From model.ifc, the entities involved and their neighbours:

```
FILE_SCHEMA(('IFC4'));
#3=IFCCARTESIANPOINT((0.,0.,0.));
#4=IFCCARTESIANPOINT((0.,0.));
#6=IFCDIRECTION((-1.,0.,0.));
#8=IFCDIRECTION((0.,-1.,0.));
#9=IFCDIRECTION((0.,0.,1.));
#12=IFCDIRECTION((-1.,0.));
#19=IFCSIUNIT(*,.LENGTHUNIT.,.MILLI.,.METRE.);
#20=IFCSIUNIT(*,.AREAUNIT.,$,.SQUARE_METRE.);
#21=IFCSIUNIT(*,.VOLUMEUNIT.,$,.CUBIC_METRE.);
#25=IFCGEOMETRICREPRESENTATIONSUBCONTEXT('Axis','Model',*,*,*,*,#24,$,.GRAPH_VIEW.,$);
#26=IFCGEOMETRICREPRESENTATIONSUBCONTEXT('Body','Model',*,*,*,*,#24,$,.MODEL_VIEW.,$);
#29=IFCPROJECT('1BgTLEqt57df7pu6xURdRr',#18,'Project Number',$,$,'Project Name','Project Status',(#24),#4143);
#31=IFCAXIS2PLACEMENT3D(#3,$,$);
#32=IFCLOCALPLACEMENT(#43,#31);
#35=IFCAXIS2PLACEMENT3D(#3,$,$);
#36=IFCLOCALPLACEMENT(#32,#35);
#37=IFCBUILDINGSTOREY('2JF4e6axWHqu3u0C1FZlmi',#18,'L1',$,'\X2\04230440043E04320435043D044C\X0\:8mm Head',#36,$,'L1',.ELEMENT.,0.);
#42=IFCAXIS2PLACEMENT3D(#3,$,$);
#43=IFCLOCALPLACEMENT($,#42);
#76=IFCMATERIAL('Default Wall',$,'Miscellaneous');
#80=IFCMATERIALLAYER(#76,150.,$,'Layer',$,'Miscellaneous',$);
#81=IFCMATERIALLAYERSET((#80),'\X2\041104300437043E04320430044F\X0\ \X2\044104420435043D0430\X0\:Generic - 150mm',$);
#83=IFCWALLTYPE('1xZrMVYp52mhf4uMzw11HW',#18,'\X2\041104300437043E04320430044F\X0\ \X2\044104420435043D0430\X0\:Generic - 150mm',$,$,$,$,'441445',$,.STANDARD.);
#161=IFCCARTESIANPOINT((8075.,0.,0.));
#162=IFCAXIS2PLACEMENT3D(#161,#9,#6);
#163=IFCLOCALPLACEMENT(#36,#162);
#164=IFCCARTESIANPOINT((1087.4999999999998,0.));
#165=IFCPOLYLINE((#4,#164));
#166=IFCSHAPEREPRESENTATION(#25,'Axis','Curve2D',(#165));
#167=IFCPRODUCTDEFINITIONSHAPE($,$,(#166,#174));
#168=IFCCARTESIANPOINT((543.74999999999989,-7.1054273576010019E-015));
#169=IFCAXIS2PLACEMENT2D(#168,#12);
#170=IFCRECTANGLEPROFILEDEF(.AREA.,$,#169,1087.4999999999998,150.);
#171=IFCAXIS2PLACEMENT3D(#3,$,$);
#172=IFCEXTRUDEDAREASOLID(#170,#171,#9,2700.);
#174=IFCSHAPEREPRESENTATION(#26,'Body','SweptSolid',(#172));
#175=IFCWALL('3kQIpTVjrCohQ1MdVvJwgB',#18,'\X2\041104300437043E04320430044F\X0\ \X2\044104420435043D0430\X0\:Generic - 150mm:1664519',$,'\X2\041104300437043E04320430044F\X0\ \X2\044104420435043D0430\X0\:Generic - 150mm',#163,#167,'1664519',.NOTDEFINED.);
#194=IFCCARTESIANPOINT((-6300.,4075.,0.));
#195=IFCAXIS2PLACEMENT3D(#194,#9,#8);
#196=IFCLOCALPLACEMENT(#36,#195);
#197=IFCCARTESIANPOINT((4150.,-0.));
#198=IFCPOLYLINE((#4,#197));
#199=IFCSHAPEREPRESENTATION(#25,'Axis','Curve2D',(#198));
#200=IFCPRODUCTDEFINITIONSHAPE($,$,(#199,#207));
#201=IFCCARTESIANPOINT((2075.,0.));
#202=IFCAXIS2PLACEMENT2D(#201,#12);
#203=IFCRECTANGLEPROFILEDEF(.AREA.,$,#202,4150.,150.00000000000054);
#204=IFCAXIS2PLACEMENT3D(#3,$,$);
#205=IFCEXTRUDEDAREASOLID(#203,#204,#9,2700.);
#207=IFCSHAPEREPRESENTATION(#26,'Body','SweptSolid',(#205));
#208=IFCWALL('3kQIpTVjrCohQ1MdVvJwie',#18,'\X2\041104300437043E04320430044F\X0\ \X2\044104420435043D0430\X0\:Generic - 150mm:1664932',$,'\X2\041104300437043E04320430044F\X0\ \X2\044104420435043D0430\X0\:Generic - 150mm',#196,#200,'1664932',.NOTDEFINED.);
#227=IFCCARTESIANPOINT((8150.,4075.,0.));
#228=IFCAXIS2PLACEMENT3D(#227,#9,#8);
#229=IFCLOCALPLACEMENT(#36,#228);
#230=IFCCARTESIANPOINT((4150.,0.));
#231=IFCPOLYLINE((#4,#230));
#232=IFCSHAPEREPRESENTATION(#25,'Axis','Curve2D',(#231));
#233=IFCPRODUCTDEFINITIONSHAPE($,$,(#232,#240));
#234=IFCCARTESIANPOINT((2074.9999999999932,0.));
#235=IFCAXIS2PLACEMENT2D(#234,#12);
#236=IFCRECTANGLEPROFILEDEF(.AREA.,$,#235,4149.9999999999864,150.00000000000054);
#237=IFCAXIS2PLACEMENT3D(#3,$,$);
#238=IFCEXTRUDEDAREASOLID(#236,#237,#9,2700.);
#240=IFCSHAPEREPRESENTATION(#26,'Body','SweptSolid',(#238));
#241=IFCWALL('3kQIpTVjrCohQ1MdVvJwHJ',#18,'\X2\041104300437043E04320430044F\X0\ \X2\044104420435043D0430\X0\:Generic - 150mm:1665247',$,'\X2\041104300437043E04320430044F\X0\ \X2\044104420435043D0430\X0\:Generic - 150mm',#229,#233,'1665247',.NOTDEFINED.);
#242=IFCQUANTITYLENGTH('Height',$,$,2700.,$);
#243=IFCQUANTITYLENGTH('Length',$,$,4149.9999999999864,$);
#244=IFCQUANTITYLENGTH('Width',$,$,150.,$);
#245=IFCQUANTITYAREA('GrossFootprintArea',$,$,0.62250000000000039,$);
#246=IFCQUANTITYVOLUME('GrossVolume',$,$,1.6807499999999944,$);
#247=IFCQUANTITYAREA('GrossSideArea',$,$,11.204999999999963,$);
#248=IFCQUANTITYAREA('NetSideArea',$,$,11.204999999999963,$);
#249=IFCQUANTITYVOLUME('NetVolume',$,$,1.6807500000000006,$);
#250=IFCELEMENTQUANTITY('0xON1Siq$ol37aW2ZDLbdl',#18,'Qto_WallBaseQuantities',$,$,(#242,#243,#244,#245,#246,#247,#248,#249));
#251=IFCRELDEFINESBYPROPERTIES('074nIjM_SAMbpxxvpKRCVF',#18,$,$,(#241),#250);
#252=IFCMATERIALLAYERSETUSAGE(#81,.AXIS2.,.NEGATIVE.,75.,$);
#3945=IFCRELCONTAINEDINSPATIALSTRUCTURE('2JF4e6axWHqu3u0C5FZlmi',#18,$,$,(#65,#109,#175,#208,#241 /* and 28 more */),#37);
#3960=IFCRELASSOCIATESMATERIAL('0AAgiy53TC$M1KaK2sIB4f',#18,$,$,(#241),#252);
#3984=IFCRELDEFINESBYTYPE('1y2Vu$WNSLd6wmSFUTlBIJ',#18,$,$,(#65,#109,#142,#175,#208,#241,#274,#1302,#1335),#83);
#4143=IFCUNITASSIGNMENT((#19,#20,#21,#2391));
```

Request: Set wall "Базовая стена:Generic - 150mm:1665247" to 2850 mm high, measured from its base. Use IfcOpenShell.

```python
import ifcopenshell
import ifcopenshell.api.pset
import ifcopenshell.geom
import ifcopenshell.util.element
import ifcopenshell.util.representation
import ifcopenshell.util.shape
import ifcopenshell.util.unit

model = ifcopenshell.open("model.ifc")
unit_scale = ifcopenshell.util.unit.calculate_unit_scale(model)
area_scale = ifcopenshell.util.unit.calculate_unit_scale(model, "AREAUNIT")
volume_scale = ifcopenshell.util.unit.calculate_unit_scale(model, "VOLUMEUNIT")
settings = ifcopenshell.geom.settings()


def volume(element):
    """Net volume in cubic metres, openings subtracted."""
    shape = ifcopenshell.geom.create_shape(settings, element)
    return ifcopenshell.util.shape.get_volume(shape.geometry)


wall = model.by_guid("3kQIpTVjrCohQ1MdVvJwHJ")
before = volume(wall)

body = ifcopenshell.util.representation.get_representation(wall, "Model", "Body")
solid = body.Items[0]
old_height = solid.Depth
solid.Depth = 2.85 / unit_scale
after = volume(wall)
thickness = 0.15  # wall thickness in metres

# Update the stored height, areas and volumes.
qto = model.by_id(ifcopenshell.util.element.get_pset(wall, "Qto_WallBaseQuantities", should_inherit=False)["id"])
ifcopenshell.api.pset.edit_qto(model, qto=qto, properties={
    "Height": solid.Depth,
    "GrossVolume": ifcopenshell.util.element.get_pset(wall, "Qto_WallBaseQuantities", "GrossVolume") * solid.Depth / old_height,
    "GrossSideArea": ifcopenshell.util.element.get_pset(wall, "Qto_WallBaseQuantities", "GrossSideArea") * solid.Depth / old_height,
    "NetSideArea": after / thickness / area_scale,
    "NetVolume": after / volume_scale,
})

print(f"height {old_height:g} -> {solid.Depth:g}, volume {before:.3f} -> {after:.3f} m3")

model.write("model_v2.ifc")
```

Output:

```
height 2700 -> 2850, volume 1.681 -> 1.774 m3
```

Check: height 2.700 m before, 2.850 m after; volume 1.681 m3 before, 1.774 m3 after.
